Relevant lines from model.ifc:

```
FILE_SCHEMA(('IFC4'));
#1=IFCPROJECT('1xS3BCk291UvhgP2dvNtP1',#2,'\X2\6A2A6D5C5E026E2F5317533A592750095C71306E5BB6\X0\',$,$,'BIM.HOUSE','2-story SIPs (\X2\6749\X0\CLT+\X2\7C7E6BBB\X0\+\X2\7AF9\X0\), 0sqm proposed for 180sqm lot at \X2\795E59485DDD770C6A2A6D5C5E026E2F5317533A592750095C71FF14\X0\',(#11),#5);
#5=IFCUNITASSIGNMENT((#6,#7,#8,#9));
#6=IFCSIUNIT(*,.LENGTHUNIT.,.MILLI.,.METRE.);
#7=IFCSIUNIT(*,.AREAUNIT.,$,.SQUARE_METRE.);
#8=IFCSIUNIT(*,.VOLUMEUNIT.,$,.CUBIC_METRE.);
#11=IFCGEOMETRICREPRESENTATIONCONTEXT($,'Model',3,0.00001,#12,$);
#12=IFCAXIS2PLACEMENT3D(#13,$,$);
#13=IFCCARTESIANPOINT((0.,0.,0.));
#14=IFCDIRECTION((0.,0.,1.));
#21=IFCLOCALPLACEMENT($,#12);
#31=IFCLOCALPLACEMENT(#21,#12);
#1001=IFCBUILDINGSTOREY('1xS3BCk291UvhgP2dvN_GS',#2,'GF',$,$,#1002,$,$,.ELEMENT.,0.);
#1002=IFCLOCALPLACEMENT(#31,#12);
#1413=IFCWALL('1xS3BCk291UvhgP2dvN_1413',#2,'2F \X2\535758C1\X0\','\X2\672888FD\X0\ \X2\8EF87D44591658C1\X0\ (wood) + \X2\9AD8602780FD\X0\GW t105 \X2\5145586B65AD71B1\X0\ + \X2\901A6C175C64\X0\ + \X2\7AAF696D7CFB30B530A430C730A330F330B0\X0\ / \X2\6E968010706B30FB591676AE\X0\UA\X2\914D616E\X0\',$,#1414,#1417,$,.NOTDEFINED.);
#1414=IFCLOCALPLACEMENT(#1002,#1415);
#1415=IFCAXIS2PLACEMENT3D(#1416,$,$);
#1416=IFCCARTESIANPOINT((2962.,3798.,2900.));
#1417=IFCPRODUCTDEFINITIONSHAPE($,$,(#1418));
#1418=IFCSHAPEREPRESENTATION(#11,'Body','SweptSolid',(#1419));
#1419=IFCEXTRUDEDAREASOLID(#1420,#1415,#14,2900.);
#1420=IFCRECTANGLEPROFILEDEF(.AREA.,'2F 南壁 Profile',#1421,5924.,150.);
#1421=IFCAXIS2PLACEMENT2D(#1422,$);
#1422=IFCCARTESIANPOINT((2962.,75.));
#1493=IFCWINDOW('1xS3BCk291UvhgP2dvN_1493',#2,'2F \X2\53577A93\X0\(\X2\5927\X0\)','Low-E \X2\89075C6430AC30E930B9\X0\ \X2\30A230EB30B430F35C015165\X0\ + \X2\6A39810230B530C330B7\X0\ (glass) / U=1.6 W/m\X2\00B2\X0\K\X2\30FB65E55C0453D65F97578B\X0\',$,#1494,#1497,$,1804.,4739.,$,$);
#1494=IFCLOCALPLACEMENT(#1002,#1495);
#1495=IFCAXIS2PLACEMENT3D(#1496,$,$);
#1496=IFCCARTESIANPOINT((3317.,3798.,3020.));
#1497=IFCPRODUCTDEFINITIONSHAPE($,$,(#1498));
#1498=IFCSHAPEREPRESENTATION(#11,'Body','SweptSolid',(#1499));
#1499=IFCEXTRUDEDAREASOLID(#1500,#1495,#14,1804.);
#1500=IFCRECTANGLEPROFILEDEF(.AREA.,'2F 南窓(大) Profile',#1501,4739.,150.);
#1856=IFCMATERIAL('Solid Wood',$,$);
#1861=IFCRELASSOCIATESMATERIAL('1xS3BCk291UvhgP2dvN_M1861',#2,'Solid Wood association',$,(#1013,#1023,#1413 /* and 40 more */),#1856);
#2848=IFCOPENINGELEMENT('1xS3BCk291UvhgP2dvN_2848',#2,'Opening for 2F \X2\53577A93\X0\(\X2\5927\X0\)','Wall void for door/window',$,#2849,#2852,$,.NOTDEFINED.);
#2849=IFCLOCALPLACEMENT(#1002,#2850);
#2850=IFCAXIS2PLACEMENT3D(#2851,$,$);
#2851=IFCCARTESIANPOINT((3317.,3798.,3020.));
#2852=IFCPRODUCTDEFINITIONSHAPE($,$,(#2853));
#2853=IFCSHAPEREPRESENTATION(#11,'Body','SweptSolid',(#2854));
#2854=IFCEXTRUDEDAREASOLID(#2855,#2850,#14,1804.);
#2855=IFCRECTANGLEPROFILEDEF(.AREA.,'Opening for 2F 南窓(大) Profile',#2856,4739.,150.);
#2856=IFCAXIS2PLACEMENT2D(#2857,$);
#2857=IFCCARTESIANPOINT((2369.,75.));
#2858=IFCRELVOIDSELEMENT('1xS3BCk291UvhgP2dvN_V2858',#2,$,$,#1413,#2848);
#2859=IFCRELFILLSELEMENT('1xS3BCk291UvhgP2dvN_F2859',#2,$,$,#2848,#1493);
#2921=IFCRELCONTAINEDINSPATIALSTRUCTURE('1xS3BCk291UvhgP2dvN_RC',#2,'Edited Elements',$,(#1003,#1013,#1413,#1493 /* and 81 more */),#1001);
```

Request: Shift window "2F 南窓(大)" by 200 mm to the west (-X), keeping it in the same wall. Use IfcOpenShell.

```python
import ifcopenshell
import ifcopenshell.api.geometry
import ifcopenshell.util.placement

model = ifcopenshell.open("model.ifc")

window = model.by_guid("1xS3BCk291UvhgP2dvN_1493")
opening = window.FillsVoids[0].RelatingOpeningElement
wall = opening.VoidsElements[0].RelatingBuildingElement

wall_matrix = ifcopenshell.util.placement.get_local_placement(wall.ObjectPlacement)
shift = wall_matrix[:3, 0] * -200.0
before = ifcopenshell.util.placement.get_local_placement(window.ObjectPlacement)[:3, 3].copy()

# The window is not placed relative to its opening, so move both.
for product in (opening, window):
    matrix = ifcopenshell.util.placement.get_local_placement(product.ObjectPlacement)
    matrix[:3, 3] += shift
    ifcopenshell.api.geometry.edit_object_placement(model, product=product, matrix=matrix, is_si=False)

after = ifcopenshell.util.placement.get_local_placement(window.ObjectPlacement)[:3, 3]
print("window moved by", (after - before).round(3) + 0.0)

model.write("model_rev.ifc")
```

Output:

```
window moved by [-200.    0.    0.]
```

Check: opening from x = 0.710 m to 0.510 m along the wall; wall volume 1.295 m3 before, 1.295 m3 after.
